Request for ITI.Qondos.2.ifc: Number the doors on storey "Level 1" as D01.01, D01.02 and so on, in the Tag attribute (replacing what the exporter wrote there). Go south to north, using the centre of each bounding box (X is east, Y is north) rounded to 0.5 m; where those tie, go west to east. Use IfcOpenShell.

First a look at what the model holds.

```python
import ifcopenshell
import ifcopenshell.util.element
import ifcopenshell.util.placement

model = ifcopenshell.open("ITI.Qondos.2.ifc")
print(model.schema)
storey = next(s for s in model.by_type("IfcBuildingStorey") if s.Name == "Level 1")
doors = [e for e in ifcopenshell.util.element.get_decomposition(storey) if e.is_a("IfcDoor")]
for e in sorted(doors, key=lambda e: e.id()):
    origin = ifcopenshell.util.placement.get_local_placement(e.ObjectPlacement)[:3, 3]
    print(e.id(), e.Tag, e.Name, origin.round(2) + 0.0, sep=" | ")
```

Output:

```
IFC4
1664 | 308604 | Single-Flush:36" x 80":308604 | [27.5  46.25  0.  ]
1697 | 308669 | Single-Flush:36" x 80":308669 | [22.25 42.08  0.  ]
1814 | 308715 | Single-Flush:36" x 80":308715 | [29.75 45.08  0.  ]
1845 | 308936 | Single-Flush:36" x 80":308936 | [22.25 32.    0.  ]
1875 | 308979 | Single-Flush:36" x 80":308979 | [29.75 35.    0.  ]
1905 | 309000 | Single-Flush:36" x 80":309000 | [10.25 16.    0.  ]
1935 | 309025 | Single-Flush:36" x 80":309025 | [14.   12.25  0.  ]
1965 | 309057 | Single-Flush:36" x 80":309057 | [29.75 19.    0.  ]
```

```python
import ifcopenshell
import ifcopenshell.geom
import ifcopenshell.util.element
import ifcopenshell.util.shape

model = ifcopenshell.open("ITI.Qondos.2.ifc")
settings = ifcopenshell.geom.settings()
settings.set("use-world-coords", True)


def centre(element):
    shape = ifcopenshell.geom.create_shape(settings, element)
    return ifcopenshell.util.shape.get_bbox_centroid(shape.geometry)


storey = next(s for s in model.by_type("IfcBuildingStorey") if s.Name == "Level 1")
doors = [e for e in ifcopenshell.util.element.get_decomposition(storey) if e.is_a("IfcDoor")]

# Insertion points can sit at a corner or the storey origin, so sort by the geometry (in metres).
centres = {e: centre(e) for e in doors}
doors.sort(key=lambda e: (round(centres[e][1] / 0.5), centres[e][0]))

for i, e in enumerate(doors, start=1):
    number = f"D01.{i:02d}"
    e.Tag = number
    print(e.id(), number)

model.write("ITI.Qondos.2_rev.ifc")
```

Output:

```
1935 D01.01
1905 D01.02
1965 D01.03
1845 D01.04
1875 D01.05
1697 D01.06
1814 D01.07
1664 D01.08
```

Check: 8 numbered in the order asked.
